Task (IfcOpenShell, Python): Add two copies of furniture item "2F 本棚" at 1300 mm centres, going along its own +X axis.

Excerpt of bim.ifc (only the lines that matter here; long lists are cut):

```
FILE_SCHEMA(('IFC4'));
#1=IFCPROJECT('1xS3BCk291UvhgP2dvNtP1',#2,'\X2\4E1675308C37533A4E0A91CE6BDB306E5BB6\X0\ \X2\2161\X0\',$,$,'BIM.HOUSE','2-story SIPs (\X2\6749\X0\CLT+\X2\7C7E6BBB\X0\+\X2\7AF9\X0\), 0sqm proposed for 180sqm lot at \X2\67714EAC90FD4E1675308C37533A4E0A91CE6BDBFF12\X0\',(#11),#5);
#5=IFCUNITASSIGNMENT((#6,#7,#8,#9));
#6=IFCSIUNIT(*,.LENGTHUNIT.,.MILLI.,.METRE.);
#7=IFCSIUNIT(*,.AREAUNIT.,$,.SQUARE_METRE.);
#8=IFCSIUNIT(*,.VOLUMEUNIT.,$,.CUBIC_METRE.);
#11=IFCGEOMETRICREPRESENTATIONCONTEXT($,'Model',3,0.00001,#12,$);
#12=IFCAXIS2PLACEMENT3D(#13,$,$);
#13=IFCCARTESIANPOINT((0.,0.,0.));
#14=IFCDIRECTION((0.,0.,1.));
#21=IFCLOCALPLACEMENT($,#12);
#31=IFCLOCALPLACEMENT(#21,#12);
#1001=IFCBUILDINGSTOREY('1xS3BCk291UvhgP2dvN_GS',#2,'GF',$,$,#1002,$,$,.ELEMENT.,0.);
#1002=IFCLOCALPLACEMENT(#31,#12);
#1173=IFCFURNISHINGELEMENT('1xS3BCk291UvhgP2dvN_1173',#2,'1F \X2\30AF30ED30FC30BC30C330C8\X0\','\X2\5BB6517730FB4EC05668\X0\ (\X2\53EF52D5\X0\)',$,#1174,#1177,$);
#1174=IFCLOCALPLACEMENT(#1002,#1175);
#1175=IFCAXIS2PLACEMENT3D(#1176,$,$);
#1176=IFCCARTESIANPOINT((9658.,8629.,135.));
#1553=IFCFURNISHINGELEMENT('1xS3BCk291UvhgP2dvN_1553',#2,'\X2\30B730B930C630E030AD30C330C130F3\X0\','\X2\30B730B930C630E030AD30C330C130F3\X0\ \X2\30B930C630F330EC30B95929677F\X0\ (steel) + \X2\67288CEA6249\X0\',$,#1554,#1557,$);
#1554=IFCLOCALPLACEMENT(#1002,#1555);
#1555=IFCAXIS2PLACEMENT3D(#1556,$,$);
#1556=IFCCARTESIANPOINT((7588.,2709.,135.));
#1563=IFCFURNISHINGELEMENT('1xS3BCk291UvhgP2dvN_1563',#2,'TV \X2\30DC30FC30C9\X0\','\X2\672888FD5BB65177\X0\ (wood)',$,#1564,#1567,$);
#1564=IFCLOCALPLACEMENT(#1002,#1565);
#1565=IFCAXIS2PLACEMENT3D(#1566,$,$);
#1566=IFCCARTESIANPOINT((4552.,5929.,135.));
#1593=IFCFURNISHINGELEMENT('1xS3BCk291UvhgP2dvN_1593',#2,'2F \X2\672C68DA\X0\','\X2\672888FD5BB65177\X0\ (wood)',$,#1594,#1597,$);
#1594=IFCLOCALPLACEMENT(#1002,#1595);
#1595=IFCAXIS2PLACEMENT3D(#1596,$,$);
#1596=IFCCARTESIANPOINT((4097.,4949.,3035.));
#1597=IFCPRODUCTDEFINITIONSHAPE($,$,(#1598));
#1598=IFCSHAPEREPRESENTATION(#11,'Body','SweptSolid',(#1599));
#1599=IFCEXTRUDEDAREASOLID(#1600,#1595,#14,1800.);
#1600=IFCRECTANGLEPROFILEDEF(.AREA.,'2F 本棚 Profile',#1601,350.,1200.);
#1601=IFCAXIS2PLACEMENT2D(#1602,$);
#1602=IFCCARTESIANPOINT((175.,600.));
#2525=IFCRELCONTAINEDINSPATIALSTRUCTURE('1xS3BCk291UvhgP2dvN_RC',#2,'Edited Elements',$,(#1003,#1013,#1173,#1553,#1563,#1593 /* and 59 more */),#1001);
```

```python
import ifcopenshell
import ifcopenshell.api.geometry
import ifcopenshell.api.root
import ifcopenshell.util.element
import ifcopenshell.util.placement

model = ifcopenshell.open("bim.ifc")


def reuse_history(source, copy):
    """copy_class also copies each property set's owner history, people and application; keep the originals."""
    for rel in copy.IsDefinedBy:
        if rel.is_a("IfcRelDefinesByProperties") and (history := rel.RelatingPropertyDefinition.OwnerHistory):
            rel.RelatingPropertyDefinition.OwnerHistory = source.OwnerHistory
            ifcopenshell.util.element.remove_deep2(model, history)


source = model.by_guid("1xS3BCk291UvhgP2dvN_1593")
base = ifcopenshell.util.placement.get_local_placement(source.ObjectPlacement)
step = base[:3, 0] * 1300.0

for i in range(1, 3):
    copy = ifcopenshell.api.root.copy_class(model, product=source)
    copy.Representation = ifcopenshell.util.element.copy_deep(
        model, source.Representation, exclude=["IfcGeometricRepresentationContext", "IfcRepresentationMap"]
    )
    reuse_history(source, copy)
    matrix = base.copy()
    matrix[:3, 3] += i * step
    print("added at", matrix[:3, 3].round(3) + 0.0)
    ifcopenshell.api.geometry.edit_object_placement(model, product=copy, matrix=matrix, is_si=False)

model.write("bim-out.ifc")
```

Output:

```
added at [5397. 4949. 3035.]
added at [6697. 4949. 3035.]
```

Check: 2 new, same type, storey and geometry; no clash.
